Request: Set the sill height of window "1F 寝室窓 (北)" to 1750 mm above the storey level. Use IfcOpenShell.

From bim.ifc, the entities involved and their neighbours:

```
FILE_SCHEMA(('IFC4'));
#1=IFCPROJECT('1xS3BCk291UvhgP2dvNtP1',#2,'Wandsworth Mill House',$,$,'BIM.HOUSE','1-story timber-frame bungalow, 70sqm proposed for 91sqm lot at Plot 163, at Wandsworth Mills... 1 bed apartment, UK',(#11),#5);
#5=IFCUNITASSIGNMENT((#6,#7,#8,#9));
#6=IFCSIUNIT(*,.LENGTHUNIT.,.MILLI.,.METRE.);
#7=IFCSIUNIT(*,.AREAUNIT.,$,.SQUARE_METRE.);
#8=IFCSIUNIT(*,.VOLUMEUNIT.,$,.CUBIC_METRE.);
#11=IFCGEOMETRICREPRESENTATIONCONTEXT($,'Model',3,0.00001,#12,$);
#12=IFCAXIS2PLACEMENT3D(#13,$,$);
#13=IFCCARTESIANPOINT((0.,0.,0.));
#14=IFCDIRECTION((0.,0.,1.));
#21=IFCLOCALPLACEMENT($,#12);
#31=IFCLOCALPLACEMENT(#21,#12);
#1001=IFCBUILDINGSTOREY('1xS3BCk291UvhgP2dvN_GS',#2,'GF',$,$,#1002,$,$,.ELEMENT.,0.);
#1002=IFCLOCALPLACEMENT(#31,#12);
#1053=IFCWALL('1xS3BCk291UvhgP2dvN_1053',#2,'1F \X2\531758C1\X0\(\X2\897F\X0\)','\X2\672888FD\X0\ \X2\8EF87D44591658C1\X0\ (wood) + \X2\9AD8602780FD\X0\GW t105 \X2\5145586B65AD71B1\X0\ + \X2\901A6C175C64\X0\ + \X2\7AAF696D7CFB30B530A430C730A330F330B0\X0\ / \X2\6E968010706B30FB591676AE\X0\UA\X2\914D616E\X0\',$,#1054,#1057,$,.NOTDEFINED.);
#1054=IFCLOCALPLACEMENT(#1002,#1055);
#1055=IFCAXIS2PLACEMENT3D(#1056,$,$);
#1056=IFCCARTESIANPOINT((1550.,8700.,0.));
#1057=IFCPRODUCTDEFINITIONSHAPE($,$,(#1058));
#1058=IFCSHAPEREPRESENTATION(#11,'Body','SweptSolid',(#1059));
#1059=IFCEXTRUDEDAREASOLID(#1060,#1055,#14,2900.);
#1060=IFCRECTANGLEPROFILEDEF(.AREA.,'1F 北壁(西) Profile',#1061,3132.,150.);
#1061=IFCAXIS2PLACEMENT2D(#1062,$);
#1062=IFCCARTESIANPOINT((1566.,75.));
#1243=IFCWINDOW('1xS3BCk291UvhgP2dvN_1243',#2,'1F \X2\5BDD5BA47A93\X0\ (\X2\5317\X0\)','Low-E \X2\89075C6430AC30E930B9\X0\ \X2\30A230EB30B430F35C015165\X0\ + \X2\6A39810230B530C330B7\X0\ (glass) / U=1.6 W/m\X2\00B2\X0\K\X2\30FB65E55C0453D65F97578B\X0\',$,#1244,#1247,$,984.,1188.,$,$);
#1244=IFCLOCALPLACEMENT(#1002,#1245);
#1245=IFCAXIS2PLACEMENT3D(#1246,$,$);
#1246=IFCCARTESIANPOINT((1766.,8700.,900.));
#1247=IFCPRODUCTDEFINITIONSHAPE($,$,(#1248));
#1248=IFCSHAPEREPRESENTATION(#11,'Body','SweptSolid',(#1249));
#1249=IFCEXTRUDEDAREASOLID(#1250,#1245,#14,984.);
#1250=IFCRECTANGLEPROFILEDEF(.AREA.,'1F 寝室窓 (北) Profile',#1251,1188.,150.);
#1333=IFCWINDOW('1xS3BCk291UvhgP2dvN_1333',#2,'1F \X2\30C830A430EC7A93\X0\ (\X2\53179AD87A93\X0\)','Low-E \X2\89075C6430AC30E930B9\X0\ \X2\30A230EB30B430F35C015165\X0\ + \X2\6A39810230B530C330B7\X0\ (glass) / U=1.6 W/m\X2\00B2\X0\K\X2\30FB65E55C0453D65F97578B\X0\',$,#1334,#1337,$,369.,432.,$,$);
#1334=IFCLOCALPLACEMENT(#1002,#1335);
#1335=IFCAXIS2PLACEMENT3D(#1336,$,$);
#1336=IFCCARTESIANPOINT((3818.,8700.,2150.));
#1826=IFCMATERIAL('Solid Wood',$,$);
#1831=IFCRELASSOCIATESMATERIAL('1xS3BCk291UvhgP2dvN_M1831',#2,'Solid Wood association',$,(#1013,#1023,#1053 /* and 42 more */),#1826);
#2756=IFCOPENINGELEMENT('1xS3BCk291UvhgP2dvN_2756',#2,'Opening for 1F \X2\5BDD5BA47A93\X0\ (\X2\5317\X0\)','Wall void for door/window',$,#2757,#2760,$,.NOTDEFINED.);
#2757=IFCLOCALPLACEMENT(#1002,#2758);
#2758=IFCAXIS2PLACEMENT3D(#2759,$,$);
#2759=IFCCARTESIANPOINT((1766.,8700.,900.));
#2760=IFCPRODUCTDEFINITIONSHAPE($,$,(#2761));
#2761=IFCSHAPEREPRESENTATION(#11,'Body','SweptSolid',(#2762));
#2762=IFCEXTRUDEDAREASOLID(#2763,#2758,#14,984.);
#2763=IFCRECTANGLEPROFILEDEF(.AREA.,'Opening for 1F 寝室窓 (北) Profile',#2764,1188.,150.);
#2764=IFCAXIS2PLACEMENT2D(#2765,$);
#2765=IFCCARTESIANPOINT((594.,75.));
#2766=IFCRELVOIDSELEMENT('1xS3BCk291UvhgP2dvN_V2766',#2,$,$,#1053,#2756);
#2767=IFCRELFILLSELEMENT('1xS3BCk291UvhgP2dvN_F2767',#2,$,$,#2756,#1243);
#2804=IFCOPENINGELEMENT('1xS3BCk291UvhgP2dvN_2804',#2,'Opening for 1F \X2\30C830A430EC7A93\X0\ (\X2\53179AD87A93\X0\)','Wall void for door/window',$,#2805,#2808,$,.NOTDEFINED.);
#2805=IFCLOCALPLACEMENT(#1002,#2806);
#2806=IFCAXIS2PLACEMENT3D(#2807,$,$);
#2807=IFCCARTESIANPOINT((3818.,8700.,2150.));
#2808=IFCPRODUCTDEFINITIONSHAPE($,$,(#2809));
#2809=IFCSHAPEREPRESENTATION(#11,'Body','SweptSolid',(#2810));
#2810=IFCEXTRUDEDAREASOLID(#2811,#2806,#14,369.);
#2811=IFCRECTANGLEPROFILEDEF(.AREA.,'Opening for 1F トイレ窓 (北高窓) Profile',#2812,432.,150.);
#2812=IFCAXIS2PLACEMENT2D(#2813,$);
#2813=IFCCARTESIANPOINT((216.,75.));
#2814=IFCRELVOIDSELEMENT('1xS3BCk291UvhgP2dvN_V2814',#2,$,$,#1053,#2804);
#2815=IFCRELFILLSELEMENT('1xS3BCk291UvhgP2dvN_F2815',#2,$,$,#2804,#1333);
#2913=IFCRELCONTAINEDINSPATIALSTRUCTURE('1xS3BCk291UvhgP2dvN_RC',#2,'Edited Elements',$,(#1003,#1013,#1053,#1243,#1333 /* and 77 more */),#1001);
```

```python
import numpy as np
import ifcopenshell
import ifcopenshell.api.geometry
import ifcopenshell.geom
import ifcopenshell.util.element
import ifcopenshell.util.placement
import ifcopenshell.util.shape
import ifcopenshell.util.unit

model = ifcopenshell.open("bim.ifc")
unit_scale = ifcopenshell.util.unit.calculate_unit_scale(model)

window = model.by_guid("1xS3BCk291UvhgP2dvN_1243")
opening = window.FillsVoids[0].RelatingOpeningElement
storey = ifcopenshell.util.element.get_container(window, ifc_class="IfcBuildingStorey")
level = ifcopenshell.util.placement.get_local_placement(storey.ObjectPlacement)[2, 3]

# The opening's origin need not be at the sill, so measure its lowest point.
shape = ifcopenshell.geom.create_shape(ifcopenshell.geom.settings(), opening)
bottom = ifcopenshell.util.shape.get_shape_bottom_elevation(shape, shape.geometry) / unit_scale
dz = level + 1.75 / unit_scale - bottom

shift = np.array([0.0, 0.0, dz])
# The window is not placed relative to its opening, so move both.
for product in (opening, window):
    matrix = ifcopenshell.util.placement.get_local_placement(product.ObjectPlacement)
    matrix[:3, 3] += shift
    ifcopenshell.api.geometry.edit_object_placement(model, product=product, matrix=matrix, is_si=False)

print(f"moved by {dz * unit_scale:+.3f} m")

model.write("bim_rev.ifc")
```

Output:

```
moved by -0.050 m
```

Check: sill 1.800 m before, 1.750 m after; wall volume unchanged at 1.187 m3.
